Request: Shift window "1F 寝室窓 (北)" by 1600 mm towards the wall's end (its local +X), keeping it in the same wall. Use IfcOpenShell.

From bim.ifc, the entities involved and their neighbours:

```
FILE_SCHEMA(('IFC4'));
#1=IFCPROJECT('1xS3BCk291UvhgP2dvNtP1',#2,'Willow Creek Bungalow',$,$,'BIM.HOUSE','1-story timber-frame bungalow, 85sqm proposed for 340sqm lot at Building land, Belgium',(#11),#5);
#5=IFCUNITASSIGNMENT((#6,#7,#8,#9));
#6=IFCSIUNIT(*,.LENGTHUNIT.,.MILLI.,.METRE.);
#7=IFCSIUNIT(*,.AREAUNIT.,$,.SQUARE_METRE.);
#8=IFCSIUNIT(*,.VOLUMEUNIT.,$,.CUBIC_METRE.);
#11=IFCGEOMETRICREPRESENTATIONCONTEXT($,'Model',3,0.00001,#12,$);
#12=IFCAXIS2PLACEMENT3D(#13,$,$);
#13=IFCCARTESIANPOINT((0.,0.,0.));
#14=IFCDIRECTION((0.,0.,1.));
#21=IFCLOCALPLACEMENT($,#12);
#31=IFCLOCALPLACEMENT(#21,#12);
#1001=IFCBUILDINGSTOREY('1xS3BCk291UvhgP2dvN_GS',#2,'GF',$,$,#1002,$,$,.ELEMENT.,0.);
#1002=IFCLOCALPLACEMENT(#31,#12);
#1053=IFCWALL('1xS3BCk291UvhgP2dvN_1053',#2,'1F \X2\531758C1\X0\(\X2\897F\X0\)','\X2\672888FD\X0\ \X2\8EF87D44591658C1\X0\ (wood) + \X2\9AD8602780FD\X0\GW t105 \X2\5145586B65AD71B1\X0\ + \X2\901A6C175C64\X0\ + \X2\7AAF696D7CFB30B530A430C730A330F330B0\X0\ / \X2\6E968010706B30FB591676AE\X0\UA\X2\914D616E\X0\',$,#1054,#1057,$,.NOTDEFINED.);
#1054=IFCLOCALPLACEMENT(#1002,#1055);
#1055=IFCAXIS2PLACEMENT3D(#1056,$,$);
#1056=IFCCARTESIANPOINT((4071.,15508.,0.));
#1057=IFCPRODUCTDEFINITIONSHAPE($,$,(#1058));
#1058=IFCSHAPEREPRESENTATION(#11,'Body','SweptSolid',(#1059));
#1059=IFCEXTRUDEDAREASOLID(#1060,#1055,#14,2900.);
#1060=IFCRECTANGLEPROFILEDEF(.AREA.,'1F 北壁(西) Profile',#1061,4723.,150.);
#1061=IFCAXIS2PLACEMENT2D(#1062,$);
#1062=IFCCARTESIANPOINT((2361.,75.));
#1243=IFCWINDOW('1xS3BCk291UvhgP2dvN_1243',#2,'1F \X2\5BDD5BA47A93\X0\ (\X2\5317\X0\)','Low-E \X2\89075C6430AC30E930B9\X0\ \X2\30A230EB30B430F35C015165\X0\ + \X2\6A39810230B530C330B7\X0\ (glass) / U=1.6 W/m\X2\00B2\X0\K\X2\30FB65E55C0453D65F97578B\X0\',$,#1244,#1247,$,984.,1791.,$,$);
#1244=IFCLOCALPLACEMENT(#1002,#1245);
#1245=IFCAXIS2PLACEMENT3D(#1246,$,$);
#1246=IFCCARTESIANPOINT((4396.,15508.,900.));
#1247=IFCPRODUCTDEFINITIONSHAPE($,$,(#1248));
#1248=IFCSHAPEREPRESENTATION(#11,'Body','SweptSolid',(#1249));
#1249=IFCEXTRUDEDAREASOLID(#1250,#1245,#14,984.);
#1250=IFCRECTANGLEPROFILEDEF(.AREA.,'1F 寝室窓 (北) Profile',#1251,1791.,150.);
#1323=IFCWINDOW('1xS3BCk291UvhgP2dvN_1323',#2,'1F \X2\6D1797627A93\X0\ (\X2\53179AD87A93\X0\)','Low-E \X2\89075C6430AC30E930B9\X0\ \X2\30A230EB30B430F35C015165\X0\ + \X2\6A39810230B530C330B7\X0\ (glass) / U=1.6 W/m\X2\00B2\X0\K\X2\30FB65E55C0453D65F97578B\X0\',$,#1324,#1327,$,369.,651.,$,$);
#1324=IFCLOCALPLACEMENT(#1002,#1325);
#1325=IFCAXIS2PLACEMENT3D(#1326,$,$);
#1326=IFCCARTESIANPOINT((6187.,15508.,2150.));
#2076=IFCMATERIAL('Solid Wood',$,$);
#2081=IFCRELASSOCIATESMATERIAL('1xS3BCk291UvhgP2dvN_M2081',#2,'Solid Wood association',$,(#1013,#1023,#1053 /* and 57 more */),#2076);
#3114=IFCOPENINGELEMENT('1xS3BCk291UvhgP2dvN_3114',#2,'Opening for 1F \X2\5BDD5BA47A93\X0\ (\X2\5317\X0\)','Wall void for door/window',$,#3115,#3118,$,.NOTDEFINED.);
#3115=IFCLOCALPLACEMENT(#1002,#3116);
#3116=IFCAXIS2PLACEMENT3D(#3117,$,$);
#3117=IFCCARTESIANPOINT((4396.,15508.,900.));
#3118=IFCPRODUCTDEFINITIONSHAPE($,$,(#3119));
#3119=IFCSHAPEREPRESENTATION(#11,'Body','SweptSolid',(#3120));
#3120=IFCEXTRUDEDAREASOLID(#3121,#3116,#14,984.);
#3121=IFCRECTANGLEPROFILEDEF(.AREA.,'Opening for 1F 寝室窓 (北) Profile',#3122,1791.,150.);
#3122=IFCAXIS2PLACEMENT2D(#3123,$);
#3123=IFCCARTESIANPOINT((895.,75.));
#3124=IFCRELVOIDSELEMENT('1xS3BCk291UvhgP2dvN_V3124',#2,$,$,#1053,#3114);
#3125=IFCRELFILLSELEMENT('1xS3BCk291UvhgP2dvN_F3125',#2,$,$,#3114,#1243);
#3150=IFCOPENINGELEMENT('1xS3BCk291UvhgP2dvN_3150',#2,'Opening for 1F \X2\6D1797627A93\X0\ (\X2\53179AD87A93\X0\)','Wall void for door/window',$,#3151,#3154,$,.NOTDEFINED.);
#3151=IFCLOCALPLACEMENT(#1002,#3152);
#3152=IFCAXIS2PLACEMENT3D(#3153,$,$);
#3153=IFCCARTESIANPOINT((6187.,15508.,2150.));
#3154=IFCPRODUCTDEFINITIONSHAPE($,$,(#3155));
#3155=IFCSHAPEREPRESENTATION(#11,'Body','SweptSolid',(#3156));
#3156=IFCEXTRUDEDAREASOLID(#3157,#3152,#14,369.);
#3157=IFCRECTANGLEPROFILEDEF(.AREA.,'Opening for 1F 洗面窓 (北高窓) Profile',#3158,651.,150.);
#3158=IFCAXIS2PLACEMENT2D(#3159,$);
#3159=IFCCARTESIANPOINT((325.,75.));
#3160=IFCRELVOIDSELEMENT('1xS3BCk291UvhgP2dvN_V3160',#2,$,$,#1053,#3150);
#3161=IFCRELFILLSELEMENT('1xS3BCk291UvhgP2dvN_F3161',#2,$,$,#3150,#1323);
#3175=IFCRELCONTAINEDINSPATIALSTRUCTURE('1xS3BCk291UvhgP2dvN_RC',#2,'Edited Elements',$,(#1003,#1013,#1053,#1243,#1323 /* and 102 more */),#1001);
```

```python
import ifcopenshell
import ifcopenshell.api.geometry
import ifcopenshell.util.placement
import ifcopenshell.util.unit

model = ifcopenshell.open("bim.ifc")
unit_scale = ifcopenshell.util.unit.calculate_unit_scale(model)

window = model.by_guid("1xS3BCk291UvhgP2dvN_1243")
opening = window.FillsVoids[0].RelatingOpeningElement
wall = opening.VoidsElements[0].RelatingBuildingElement

wall_matrix = ifcopenshell.util.placement.get_local_placement(wall.ObjectPlacement)
shift = wall_matrix[:3, 0] * 1.6 / unit_scale
before = ifcopenshell.util.placement.get_local_placement(window.ObjectPlacement)[:3, 3].copy()

# The window is not placed relative to its opening, so move both.
for product in (opening, window):
    matrix = ifcopenshell.util.placement.get_local_placement(product.ObjectPlacement)
    matrix[:3, 3] += shift
    ifcopenshell.api.geometry.edit_object_placement(model, product=product, matrix=matrix, is_si=False)

after = ifcopenshell.util.placement.get_local_placement(window.ObjectPlacement)[:3, 3]
print("window moved by", (after - before).round(3) + 0.0)

model.write("bim_edited.ifc")
```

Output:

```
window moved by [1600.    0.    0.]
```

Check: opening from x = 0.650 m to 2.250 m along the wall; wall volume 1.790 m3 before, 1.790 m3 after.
